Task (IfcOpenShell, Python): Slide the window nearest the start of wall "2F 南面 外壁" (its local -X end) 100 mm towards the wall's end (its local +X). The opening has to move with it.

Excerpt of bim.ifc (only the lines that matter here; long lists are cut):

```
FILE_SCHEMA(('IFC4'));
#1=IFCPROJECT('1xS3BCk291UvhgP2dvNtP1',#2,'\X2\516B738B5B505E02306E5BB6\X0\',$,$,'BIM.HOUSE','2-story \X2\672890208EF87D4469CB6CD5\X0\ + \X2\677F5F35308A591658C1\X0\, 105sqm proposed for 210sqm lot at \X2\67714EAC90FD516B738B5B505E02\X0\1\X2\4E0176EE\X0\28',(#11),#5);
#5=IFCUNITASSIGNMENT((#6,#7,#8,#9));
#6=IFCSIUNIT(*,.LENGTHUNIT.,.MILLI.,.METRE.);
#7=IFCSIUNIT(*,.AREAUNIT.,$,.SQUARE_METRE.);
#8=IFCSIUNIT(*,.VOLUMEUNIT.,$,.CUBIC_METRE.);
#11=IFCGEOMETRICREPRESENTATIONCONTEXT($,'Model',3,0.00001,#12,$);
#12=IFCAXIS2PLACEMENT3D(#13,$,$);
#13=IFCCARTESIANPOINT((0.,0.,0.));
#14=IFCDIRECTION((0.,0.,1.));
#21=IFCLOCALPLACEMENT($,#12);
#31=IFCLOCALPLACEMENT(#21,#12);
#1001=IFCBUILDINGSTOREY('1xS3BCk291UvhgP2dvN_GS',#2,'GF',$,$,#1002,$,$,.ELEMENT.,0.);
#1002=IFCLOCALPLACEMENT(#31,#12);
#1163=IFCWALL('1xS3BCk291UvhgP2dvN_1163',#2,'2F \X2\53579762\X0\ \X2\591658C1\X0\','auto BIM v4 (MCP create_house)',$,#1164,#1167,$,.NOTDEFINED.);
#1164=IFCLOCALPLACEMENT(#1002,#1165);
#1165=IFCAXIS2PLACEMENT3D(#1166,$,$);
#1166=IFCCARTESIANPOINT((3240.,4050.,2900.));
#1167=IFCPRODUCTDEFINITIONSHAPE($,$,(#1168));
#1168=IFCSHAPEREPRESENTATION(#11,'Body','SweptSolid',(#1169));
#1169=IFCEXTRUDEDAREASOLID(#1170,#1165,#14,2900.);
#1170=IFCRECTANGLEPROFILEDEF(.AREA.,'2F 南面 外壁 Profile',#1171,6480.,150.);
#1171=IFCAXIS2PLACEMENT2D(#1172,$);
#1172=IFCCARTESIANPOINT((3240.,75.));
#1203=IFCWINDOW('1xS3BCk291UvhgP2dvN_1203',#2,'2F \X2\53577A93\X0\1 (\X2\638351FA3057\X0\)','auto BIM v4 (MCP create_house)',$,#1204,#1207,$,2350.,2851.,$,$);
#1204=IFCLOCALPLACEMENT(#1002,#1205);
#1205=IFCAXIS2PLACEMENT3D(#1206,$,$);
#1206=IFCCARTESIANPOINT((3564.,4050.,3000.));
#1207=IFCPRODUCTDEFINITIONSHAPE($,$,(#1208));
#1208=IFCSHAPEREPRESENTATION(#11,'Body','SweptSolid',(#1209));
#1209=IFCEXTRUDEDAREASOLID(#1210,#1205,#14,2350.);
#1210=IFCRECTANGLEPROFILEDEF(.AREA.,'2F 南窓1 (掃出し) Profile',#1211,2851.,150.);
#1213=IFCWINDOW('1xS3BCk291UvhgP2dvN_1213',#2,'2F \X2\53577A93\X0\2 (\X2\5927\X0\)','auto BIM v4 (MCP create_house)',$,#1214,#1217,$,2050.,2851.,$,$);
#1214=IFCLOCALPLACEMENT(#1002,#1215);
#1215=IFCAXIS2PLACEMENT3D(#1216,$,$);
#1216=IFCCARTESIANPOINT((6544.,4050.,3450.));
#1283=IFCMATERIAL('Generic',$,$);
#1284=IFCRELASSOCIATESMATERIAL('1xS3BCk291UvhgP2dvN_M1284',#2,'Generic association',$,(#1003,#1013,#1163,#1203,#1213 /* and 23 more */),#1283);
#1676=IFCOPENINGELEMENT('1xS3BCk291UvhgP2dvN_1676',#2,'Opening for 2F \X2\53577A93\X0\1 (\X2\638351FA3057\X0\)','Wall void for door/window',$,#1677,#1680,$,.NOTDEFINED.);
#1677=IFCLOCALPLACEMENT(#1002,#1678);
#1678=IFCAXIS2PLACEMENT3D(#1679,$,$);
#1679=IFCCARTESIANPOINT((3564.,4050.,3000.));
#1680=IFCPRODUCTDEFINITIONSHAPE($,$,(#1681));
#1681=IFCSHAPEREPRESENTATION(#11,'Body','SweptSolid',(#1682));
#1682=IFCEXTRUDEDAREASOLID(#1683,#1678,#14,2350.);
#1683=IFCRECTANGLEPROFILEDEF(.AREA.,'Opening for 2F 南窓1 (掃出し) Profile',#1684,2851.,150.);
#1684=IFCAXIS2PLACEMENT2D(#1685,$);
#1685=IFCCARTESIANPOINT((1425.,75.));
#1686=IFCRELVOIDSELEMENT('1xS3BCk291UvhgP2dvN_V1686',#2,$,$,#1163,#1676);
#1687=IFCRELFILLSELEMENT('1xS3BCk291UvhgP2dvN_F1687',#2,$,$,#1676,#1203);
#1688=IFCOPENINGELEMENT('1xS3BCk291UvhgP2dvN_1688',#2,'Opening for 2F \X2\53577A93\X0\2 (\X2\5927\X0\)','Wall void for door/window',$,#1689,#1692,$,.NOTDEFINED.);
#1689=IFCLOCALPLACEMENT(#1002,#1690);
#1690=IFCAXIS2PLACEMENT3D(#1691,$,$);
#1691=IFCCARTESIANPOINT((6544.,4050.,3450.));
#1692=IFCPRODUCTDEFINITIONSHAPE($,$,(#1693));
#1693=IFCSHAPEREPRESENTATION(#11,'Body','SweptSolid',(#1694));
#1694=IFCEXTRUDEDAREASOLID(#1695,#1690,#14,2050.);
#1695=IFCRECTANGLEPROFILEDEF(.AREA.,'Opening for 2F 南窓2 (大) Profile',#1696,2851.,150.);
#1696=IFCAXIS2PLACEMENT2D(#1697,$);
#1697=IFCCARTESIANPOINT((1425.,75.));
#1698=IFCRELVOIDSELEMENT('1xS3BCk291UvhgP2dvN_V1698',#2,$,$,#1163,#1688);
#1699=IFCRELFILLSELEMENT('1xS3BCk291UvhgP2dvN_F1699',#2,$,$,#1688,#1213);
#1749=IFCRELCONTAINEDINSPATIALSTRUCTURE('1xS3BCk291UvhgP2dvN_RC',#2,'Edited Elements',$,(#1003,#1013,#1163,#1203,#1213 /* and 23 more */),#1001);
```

```python
import ifcopenshell
import ifcopenshell.api.geometry
import ifcopenshell.util.placement
import ifcopenshell.util.unit

model = ifcopenshell.open("bim.ifc")
unit_scale = ifcopenshell.util.unit.calculate_unit_scale(model)

window = model.by_guid("1xS3BCk291UvhgP2dvN_1203")
opening = window.FillsVoids[0].RelatingOpeningElement
wall = opening.VoidsElements[0].RelatingBuildingElement

wall_matrix = ifcopenshell.util.placement.get_local_placement(wall.ObjectPlacement)
shift = wall_matrix[:3, 0] * 0.1 / unit_scale
before = ifcopenshell.util.placement.get_local_placement(window.ObjectPlacement)[:3, 3].copy()

# The window is not placed relative to its opening, so move both.
for product in (opening, window):
    matrix = ifcopenshell.util.placement.get_local_placement(product.ObjectPlacement)
    matrix[:3, 3] += shift
    ifcopenshell.api.geometry.edit_object_placement(model, product=product, matrix=matrix, is_si=False)

after = ifcopenshell.util.placement.get_local_placement(window.ObjectPlacement)[:3, 3]
print("window moved by", (after - before).round(3) + 0.0)

model.write("bim_rev.ifc")
```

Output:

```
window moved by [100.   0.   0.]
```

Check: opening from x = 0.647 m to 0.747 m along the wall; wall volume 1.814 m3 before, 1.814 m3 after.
